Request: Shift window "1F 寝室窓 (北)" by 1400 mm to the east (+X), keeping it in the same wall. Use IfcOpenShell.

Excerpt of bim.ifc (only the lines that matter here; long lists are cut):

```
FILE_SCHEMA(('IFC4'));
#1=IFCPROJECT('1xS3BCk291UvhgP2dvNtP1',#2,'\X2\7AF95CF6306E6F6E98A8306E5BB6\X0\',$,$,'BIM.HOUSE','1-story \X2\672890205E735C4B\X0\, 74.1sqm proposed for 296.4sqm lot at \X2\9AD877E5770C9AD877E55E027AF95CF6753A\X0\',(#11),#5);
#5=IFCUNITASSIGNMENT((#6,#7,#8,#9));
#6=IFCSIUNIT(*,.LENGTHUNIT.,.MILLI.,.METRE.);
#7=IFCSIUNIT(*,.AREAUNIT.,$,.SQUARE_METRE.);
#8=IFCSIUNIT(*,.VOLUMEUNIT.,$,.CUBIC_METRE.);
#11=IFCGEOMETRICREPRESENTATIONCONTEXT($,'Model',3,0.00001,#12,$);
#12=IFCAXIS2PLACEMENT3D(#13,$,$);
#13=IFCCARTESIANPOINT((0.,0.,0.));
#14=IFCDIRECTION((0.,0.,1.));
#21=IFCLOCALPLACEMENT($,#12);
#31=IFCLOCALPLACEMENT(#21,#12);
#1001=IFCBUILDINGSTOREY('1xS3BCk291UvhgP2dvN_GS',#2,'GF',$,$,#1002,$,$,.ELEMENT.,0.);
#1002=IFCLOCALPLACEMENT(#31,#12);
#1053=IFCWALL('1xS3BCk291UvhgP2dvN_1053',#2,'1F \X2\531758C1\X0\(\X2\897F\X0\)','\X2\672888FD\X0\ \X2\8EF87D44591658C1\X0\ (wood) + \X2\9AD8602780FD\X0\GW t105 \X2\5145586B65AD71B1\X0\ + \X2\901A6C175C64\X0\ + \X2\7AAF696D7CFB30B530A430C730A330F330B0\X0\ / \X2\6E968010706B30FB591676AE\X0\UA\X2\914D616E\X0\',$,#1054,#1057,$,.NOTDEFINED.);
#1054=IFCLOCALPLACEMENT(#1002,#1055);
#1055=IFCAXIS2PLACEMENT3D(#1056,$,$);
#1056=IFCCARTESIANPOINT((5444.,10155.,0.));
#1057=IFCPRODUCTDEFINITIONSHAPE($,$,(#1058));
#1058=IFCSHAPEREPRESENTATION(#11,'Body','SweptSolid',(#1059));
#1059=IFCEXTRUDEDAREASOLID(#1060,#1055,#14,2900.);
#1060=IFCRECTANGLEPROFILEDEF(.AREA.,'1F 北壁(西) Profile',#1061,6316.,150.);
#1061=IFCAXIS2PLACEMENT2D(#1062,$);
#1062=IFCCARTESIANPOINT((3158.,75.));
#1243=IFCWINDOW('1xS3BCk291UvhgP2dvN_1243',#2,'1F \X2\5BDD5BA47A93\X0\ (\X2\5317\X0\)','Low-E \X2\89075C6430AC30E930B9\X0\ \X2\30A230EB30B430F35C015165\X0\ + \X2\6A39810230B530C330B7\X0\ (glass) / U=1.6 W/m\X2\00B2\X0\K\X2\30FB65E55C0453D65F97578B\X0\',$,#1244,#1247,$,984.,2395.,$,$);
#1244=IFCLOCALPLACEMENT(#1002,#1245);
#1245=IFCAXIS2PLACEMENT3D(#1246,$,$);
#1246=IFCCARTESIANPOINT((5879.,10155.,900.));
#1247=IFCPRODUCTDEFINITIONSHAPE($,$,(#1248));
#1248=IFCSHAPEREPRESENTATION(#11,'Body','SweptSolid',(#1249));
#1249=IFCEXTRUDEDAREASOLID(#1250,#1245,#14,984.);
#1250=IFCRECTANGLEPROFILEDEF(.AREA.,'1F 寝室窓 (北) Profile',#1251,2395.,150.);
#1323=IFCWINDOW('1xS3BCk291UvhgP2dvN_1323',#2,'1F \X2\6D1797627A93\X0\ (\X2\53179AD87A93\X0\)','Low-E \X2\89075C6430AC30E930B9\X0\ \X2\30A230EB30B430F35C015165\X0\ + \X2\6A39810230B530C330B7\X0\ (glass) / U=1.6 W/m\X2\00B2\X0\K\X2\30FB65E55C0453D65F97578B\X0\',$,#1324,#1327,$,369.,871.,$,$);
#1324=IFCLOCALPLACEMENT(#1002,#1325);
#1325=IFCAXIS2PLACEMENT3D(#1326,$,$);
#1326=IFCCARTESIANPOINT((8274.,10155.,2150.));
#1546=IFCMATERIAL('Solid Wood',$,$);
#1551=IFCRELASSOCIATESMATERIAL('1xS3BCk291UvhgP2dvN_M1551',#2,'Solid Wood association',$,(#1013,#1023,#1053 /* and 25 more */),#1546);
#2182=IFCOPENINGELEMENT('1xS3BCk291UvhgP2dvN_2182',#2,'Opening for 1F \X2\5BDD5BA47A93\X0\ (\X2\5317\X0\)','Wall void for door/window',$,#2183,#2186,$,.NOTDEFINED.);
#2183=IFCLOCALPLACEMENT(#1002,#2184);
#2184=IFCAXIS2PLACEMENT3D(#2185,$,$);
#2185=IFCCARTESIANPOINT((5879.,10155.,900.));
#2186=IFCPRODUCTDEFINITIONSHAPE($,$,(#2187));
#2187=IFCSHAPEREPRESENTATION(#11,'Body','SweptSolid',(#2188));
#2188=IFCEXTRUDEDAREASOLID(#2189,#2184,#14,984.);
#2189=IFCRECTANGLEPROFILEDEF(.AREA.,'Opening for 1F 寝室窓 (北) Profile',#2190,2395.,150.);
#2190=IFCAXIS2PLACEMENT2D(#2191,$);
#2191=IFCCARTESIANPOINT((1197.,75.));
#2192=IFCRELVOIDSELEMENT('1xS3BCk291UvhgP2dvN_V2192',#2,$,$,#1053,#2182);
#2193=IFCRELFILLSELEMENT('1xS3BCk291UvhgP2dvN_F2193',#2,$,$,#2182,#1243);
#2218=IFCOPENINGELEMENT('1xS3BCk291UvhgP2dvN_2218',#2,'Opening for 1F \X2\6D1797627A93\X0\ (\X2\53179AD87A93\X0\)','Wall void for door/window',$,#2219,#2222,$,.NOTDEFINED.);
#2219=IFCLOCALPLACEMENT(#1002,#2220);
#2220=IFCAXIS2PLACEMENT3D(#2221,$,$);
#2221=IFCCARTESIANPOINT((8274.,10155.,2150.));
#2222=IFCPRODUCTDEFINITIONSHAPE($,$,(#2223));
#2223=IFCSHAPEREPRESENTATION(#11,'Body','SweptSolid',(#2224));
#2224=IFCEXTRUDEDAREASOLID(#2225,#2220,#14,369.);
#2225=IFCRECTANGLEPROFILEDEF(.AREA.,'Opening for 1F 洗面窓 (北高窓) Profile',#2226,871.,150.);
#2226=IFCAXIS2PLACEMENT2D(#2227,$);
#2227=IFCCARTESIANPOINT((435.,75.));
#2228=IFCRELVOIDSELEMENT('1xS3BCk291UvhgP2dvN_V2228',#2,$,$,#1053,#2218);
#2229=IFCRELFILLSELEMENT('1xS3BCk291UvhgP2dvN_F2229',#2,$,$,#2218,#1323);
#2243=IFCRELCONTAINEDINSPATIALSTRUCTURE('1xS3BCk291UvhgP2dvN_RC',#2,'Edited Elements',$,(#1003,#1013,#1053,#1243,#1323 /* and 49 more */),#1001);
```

```python
import ifcopenshell
import ifcopenshell.api.geometry
import ifcopenshell.util.placement

model = ifcopenshell.open("bim.ifc")

window = model.by_guid("1xS3BCk291UvhgP2dvN_1243")
opening = window.FillsVoids[0].RelatingOpeningElement
wall = opening.VoidsElements[0].RelatingBuildingElement

wall_matrix = ifcopenshell.util.placement.get_local_placement(wall.ObjectPlacement)
shift = wall_matrix[:3, 0] * 1400.0
before = ifcopenshell.util.placement.get_local_placement(window.ObjectPlacement)[:3, 3].copy()

# The window is not placed relative to its opening, so move both.
for product in (opening, window):
    matrix = ifcopenshell.util.placement.get_local_placement(product.ObjectPlacement)
    matrix[:3, 3] += shift
    ifcopenshell.api.geometry.edit_object_placement(model, product=product, matrix=matrix, is_si=False)

after = ifcopenshell.util.placement.get_local_placement(window.ObjectPlacement)[:3, 3]
print("window moved by", (after - before).round(3) + 0.0)

model.write("bim-out.ifc")
```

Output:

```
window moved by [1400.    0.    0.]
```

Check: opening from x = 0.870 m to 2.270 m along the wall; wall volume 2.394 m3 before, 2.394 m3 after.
